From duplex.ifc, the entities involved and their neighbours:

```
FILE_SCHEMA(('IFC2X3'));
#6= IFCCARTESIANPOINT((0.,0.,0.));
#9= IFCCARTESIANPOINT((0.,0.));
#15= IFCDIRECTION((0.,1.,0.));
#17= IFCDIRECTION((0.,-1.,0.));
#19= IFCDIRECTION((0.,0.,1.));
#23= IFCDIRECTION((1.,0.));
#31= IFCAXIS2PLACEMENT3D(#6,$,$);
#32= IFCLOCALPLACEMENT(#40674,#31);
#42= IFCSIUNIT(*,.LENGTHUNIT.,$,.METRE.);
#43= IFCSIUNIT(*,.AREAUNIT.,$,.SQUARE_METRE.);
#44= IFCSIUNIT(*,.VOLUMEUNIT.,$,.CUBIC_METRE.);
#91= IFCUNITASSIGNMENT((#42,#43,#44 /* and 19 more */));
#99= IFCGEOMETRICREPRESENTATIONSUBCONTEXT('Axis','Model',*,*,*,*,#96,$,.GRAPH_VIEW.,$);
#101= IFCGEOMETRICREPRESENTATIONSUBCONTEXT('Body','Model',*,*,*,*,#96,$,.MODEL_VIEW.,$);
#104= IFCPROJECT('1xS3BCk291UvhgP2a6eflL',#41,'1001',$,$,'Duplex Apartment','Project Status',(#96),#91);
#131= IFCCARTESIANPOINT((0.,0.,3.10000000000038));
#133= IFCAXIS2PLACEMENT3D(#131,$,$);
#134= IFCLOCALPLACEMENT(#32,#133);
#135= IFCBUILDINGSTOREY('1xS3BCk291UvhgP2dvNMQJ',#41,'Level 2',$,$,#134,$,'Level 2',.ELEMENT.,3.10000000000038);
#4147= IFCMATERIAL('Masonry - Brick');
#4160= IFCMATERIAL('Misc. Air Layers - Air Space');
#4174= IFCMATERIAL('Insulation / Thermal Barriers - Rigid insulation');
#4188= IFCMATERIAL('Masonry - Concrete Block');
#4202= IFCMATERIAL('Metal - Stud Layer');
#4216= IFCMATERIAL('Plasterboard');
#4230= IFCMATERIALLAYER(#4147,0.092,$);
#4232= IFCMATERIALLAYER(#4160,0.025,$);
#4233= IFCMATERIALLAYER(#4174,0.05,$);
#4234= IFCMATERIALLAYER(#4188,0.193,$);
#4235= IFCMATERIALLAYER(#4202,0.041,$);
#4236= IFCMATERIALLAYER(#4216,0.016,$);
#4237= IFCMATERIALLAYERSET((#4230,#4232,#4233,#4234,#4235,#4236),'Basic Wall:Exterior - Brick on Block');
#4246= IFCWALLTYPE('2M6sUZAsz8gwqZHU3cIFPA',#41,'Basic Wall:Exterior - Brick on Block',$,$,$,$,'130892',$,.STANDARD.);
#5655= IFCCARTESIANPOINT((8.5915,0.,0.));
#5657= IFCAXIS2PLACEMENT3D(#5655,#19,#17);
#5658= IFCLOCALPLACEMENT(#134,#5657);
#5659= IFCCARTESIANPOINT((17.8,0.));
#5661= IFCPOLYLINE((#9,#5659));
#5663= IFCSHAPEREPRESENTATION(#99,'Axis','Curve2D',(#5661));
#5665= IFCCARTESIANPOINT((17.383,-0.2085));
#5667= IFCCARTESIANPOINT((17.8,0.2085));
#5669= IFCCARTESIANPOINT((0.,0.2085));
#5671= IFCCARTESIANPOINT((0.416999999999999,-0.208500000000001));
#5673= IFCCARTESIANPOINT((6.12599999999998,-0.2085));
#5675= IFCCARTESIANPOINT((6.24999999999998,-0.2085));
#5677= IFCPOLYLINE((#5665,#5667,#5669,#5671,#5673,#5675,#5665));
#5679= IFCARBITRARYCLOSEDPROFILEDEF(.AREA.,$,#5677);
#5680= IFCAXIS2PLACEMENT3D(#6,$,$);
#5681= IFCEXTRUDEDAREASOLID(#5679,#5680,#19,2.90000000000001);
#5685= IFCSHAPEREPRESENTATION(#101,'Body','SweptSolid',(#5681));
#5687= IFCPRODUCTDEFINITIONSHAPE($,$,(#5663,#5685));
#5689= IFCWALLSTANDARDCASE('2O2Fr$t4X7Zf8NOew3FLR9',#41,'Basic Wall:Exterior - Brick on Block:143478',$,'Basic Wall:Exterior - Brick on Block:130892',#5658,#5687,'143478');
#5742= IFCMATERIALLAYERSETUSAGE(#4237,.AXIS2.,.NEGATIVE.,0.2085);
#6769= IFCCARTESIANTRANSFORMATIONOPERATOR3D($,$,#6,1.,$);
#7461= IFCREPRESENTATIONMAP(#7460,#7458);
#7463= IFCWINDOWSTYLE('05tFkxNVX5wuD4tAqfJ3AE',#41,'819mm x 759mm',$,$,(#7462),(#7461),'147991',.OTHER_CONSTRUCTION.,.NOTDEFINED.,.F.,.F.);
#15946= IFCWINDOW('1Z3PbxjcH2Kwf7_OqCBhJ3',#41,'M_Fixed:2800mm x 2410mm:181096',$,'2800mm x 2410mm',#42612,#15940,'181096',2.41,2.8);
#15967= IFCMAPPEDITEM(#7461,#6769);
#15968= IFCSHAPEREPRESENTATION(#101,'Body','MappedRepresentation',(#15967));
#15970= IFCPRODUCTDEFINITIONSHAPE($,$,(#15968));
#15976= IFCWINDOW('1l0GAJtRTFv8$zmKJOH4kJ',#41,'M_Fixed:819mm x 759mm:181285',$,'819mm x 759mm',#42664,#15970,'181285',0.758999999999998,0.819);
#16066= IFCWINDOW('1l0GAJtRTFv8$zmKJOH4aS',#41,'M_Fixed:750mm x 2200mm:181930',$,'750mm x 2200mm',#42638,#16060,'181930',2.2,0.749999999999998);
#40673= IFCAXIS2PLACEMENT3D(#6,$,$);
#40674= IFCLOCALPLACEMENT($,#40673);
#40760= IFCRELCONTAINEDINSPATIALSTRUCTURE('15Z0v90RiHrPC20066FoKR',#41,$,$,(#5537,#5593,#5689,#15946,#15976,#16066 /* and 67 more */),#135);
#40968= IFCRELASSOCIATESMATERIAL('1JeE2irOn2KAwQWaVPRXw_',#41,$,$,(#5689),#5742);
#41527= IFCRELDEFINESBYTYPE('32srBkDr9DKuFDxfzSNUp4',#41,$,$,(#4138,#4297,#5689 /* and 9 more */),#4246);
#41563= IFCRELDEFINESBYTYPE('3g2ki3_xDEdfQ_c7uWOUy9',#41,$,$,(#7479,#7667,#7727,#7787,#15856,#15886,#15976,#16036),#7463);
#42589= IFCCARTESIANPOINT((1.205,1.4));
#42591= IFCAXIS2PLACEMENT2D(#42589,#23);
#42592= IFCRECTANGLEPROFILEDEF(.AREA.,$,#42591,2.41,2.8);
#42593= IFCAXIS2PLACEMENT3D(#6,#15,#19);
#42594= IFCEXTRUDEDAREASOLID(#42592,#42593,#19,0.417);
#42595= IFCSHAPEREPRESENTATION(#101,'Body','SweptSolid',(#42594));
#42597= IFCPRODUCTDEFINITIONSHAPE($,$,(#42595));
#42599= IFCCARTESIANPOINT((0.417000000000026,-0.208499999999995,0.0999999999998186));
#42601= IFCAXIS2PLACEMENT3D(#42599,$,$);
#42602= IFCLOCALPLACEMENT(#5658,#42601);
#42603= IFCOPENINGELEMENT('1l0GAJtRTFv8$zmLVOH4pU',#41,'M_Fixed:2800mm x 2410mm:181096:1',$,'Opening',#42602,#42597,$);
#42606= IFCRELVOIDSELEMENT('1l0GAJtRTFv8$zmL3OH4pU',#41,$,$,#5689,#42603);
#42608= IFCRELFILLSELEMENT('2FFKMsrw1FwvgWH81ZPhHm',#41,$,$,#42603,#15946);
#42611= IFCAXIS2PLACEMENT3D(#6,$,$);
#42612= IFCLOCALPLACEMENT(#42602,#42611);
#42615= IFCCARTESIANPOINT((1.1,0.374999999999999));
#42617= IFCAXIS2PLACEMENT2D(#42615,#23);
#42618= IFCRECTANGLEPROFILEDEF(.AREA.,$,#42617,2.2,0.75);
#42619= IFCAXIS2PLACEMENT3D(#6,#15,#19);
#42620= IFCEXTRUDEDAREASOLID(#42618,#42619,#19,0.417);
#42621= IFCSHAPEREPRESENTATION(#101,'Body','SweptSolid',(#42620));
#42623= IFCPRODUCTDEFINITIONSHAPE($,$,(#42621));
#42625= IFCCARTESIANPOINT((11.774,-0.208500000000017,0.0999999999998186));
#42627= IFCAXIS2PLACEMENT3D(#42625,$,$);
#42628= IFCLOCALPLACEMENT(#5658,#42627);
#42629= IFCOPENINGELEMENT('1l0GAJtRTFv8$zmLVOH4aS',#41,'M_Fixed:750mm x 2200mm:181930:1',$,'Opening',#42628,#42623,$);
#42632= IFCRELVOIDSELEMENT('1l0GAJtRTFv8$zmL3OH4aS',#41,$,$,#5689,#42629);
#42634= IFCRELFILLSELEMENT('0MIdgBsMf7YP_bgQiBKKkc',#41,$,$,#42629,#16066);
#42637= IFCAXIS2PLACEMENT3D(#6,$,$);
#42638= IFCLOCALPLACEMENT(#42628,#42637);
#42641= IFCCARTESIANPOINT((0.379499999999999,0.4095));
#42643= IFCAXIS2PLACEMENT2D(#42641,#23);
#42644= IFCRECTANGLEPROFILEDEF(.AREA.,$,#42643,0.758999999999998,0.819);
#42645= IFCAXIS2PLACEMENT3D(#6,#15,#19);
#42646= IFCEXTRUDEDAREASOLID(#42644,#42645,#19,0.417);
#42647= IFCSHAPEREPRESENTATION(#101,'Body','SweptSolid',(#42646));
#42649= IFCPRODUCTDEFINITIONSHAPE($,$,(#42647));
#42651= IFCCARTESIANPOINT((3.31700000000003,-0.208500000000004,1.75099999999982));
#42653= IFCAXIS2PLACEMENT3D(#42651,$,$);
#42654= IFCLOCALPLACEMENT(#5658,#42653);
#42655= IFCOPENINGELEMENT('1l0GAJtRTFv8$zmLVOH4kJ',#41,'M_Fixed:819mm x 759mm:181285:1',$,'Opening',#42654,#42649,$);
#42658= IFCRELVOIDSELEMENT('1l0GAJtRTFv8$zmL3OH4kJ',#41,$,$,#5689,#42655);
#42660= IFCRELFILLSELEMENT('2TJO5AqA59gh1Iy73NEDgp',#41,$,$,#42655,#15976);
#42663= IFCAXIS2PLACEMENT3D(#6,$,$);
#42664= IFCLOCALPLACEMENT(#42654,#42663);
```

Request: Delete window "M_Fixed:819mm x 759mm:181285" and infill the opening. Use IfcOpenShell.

```python
import ifcopenshell
import ifcopenshell.api.feature
import ifcopenshell.api.root
import ifcopenshell.geom
import ifcopenshell.util.shape

model = ifcopenshell.open("duplex.ifc")
settings = ifcopenshell.geom.settings()


def volume(element):
    """Net volume in cubic metres, openings subtracted."""
    shape = ifcopenshell.geom.create_shape(settings, element)
    return ifcopenshell.util.shape.get_volume(shape.geometry)


window = model.by_id(15976)
opening = window.FillsVoids[0].RelatingOpeningElement
wall = opening.VoidsElements[0].RelatingBuildingElement
before = volume(wall)

ifcopenshell.api.root.remove_product(model, product=window)
ifcopenshell.api.feature.remove_feature(model, feature=opening)

after = volume(wall)

print(f"wall volume {before:.3f} -> {after:.3f} m3")

model.write("duplex-out.ifc")
```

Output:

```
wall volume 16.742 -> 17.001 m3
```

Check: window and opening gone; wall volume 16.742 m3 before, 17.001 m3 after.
